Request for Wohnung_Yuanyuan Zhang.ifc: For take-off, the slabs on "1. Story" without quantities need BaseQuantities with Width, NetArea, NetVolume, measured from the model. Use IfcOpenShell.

First a look at what the model holds.

```python
import ifcopenshell
import ifcopenshell.util.element
import ifcopenshell.util.unit

model = ifcopenshell.open("Wohnung_Yuanyuan Zhang.ifc")
print(model.schema)
for unit_type in ("LENGTHUNIT", "AREAUNIT", "VOLUMEUNIT"):
    print(unit_type, ifcopenshell.util.unit.calculate_unit_scale(model, unit_type))
storey = next(s for s in model.by_type("IfcBuildingStorey") if s.Name == "1. Story")
slabs = [e for e in ifcopenshell.util.element.get_decomposition(storey) if e.is_a("IfcSlab")]
for e in sorted(slabs, key=lambda e: e.id()):
    print(e.id(), e.is_a(), e.Name, list(ifcopenshell.util.element.get_psets(e, qtos_only=True)), sep=" | ")
```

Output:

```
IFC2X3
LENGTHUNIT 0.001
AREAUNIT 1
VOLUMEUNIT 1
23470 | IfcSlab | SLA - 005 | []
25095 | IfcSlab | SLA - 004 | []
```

```python
import ifcopenshell
import ifcopenshell.api.pset
import ifcopenshell.geom
import ifcopenshell.util.element
import ifcopenshell.util.shape
import ifcopenshell.util.unit

model = ifcopenshell.open("Wohnung_Yuanyuan Zhang.ifc")
unit_scale = ifcopenshell.util.unit.calculate_unit_scale(model)
area_scale = ifcopenshell.util.unit.calculate_unit_scale(model, "AREAUNIT")
volume_scale = ifcopenshell.util.unit.calculate_unit_scale(model, "VOLUMEUNIT")
settings = ifcopenshell.geom.settings()

storey = next(s for s in model.by_type("IfcBuildingStorey") if s.Name == "1. Story")
slabs = [e for e in ifcopenshell.util.element.get_decomposition(storey) if e.is_a("IfcSlab")]

for e in sorted(slabs, key=lambda e: e.id()):
    if ifcopenshell.util.element.get_psets(e, qtos_only=True, should_inherit=False):
        continue
    # Geometry comes back in metres, in the element's own axes.
    shape = ifcopenshell.geom.create_shape(settings, e)
    values = {
        "Width": ifcopenshell.util.shape.get_z(shape.geometry) / unit_scale,
        "NetArea": ifcopenshell.util.shape.get_footprint_area(shape.geometry) / area_scale,
        "NetVolume": ifcopenshell.util.shape.get_volume(shape.geometry) / volume_scale,
    }
    qto = ifcopenshell.api.pset.add_qto(model, product=e, name="BaseQuantities")
    ifcopenshell.api.pset.edit_qto(model, qto=qto, properties=values)
    print(e.id(), {k: round(v, 3) for k, v in values.items()})

model.write("Wohnung_Yuanyuan Zhang_v2.ifc")
```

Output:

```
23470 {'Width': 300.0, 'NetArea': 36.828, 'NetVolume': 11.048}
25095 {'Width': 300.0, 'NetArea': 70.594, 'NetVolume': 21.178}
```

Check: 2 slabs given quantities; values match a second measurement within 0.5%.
